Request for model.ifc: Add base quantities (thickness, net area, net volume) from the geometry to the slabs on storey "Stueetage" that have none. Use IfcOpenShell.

First a look at what the model holds.

```python
import ifcopenshell
import ifcopenshell.util.element
import ifcopenshell.util.unit

model = ifcopenshell.open("model.ifc")
print(model.schema)
for unit_type in ("LENGTHUNIT", "AREAUNIT", "VOLUMEUNIT"):
    print(unit_type, ifcopenshell.util.unit.calculate_unit_scale(model, unit_type))
storey = next(s for s in model.by_type("IfcBuildingStorey") if s.Name == "Stueetage")
slabs = [e for e in ifcopenshell.util.element.get_decomposition(storey) if e.is_a("IfcSlab")]
for e in sorted(slabs, key=lambda e: e.id()):
    print(e.id(), e.is_a(), e.Name, list(ifcopenshell.util.element.get_psets(e, qtos_only=True)), sep=" | ")
```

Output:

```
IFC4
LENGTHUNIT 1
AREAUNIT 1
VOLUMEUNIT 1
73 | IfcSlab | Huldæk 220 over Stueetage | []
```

```python
import ifcopenshell
import ifcopenshell.api.pset
import ifcopenshell.geom
import ifcopenshell.util.element
import ifcopenshell.util.shape
import ifcopenshell.util.unit

model = ifcopenshell.open("model.ifc")
unit_scale = ifcopenshell.util.unit.calculate_unit_scale(model)
area_scale = ifcopenshell.util.unit.calculate_unit_scale(model, "AREAUNIT")
volume_scale = ifcopenshell.util.unit.calculate_unit_scale(model, "VOLUMEUNIT")
settings = ifcopenshell.geom.settings()

storey = next(s for s in model.by_type("IfcBuildingStorey") if s.Name == "Stueetage")
slabs = [e for e in ifcopenshell.util.element.get_decomposition(storey) if e.is_a("IfcSlab")]

for e in sorted(slabs, key=lambda e: e.id()):
    if ifcopenshell.util.element.get_psets(e, qtos_only=True, should_inherit=False):
        continue
    # Geometry comes back in metres, in the element's own axes.
    shape = ifcopenshell.geom.create_shape(settings, e)
    values = {
        "Width": ifcopenshell.util.shape.get_z(shape.geometry) / unit_scale,
        "NetArea": ifcopenshell.util.shape.get_footprint_area(shape.geometry) / area_scale,
        "NetVolume": ifcopenshell.util.shape.get_volume(shape.geometry) / volume_scale,
    }
    qto = ifcopenshell.api.pset.add_qto(model, product=e, name="Qto_SlabBaseQuantities")
    ifcopenshell.api.pset.edit_qto(model, qto=qto, properties=values)
    print(e.id(), {k: round(v, 3) for k, v in values.items()})

model.write("model-out.ifc")
```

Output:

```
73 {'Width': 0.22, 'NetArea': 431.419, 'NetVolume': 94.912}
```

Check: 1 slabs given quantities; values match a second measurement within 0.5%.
